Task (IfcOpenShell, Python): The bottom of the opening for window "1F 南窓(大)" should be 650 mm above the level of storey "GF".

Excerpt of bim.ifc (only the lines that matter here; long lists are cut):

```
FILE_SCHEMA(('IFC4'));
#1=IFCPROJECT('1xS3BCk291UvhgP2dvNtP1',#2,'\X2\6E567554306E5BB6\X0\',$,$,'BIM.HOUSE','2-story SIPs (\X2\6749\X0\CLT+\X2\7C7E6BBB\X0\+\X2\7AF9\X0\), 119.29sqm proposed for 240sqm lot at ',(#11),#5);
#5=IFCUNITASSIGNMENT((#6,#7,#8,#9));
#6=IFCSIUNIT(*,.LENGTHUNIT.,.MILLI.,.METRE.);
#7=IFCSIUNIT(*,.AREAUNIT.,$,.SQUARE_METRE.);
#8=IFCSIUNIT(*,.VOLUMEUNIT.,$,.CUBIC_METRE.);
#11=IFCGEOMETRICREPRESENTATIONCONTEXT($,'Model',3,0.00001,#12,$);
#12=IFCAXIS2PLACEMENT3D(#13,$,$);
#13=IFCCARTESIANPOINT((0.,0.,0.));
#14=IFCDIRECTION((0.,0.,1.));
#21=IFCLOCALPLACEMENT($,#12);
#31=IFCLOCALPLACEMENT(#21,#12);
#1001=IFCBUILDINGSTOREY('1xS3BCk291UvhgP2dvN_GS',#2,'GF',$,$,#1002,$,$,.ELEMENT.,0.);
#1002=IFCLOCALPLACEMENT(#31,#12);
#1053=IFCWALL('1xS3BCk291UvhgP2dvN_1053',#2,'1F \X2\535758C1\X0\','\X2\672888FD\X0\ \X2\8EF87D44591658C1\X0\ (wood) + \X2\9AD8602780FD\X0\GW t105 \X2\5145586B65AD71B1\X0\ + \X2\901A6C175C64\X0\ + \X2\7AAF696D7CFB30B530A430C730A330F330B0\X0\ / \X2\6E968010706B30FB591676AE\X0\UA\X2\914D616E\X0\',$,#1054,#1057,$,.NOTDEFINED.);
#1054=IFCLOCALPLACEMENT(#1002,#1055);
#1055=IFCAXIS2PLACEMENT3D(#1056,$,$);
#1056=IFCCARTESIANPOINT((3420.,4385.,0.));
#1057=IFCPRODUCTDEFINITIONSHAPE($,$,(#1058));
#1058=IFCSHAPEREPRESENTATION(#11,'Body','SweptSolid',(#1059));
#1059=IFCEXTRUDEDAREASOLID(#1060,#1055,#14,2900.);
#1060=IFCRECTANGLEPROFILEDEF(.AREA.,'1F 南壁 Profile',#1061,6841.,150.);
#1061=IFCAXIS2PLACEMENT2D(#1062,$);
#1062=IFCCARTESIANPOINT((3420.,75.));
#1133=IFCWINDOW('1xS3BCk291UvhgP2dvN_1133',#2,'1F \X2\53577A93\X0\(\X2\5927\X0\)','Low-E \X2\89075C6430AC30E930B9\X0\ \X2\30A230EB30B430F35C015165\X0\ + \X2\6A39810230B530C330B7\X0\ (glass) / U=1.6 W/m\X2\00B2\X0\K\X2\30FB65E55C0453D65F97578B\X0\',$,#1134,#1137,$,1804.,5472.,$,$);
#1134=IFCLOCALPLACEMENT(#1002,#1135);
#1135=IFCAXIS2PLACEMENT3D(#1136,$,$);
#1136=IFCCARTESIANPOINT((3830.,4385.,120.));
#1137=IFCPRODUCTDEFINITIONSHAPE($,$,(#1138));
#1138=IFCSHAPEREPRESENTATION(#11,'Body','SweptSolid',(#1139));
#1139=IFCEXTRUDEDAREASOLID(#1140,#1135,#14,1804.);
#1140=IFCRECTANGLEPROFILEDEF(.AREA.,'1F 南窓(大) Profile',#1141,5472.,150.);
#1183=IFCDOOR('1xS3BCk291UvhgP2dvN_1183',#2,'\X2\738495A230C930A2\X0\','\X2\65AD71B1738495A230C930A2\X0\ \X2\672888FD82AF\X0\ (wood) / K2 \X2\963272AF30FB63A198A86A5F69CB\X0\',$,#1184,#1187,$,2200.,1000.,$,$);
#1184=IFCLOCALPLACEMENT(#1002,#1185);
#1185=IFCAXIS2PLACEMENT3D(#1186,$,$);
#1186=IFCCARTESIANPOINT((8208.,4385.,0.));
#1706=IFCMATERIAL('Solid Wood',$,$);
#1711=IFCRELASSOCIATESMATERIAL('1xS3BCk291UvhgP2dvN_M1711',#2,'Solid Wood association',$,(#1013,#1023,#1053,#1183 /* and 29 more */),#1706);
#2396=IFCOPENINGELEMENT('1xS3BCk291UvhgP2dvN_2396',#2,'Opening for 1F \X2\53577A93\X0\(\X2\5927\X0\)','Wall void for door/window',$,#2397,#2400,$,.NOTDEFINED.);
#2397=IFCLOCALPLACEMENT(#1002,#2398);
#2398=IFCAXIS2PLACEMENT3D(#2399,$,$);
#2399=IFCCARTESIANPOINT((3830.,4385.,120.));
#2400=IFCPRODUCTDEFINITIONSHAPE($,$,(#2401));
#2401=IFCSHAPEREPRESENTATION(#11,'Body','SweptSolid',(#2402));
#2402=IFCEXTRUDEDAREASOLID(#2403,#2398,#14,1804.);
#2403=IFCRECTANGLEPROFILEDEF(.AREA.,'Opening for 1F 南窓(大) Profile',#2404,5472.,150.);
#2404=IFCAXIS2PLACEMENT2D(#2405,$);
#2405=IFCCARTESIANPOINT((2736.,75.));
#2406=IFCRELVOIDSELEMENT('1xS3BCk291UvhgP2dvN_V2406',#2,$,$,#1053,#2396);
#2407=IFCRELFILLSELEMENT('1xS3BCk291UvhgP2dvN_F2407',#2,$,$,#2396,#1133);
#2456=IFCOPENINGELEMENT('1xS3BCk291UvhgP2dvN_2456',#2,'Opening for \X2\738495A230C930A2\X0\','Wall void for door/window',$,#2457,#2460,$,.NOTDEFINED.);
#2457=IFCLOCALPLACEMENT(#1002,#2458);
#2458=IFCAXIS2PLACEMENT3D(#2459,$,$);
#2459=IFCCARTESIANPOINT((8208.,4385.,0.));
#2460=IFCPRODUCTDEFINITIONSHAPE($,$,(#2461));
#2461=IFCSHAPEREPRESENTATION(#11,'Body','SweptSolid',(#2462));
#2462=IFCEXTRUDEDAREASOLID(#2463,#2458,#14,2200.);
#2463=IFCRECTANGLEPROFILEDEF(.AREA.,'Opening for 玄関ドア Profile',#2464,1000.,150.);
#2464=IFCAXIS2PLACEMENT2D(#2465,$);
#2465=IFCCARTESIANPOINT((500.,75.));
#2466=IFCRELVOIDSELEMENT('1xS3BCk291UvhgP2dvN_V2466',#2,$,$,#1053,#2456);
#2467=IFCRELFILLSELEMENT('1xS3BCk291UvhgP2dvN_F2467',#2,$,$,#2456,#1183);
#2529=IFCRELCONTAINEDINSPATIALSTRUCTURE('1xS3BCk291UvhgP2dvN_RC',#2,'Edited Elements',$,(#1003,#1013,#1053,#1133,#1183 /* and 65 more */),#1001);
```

```python
import numpy as np
import ifcopenshell
import ifcopenshell.api.geometry
import ifcopenshell.geom
import ifcopenshell.util.element
import ifcopenshell.util.placement
import ifcopenshell.util.shape
import ifcopenshell.util.unit

model = ifcopenshell.open("bim.ifc")
unit_scale = ifcopenshell.util.unit.calculate_unit_scale(model)

window = model.by_guid("1xS3BCk291UvhgP2dvN_1133")
opening = window.FillsVoids[0].RelatingOpeningElement
storey = ifcopenshell.util.element.get_container(window, ifc_class="IfcBuildingStorey")
level = ifcopenshell.util.placement.get_local_placement(storey.ObjectPlacement)[2, 3]

# The opening's origin need not be at the sill, so measure its lowest point.
shape = ifcopenshell.geom.create_shape(ifcopenshell.geom.settings(), opening)
bottom = ifcopenshell.util.shape.get_shape_bottom_elevation(shape, shape.geometry) / unit_scale
dz = level + 650.0 - bottom

shift = np.array([0.0, 0.0, dz])
# The window is not placed relative to its opening, so move both.
for product in (opening, window):
    matrix = ifcopenshell.util.placement.get_local_placement(product.ObjectPlacement)
    matrix[:3, 3] += shift
    ifcopenshell.api.geometry.edit_object_placement(model, product=product, matrix=matrix, is_si=False)

print(f"moved by {dz * unit_scale:+.3f} m")

model.write("bim_v2.ifc")
```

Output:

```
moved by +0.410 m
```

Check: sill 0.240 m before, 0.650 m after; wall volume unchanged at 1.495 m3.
